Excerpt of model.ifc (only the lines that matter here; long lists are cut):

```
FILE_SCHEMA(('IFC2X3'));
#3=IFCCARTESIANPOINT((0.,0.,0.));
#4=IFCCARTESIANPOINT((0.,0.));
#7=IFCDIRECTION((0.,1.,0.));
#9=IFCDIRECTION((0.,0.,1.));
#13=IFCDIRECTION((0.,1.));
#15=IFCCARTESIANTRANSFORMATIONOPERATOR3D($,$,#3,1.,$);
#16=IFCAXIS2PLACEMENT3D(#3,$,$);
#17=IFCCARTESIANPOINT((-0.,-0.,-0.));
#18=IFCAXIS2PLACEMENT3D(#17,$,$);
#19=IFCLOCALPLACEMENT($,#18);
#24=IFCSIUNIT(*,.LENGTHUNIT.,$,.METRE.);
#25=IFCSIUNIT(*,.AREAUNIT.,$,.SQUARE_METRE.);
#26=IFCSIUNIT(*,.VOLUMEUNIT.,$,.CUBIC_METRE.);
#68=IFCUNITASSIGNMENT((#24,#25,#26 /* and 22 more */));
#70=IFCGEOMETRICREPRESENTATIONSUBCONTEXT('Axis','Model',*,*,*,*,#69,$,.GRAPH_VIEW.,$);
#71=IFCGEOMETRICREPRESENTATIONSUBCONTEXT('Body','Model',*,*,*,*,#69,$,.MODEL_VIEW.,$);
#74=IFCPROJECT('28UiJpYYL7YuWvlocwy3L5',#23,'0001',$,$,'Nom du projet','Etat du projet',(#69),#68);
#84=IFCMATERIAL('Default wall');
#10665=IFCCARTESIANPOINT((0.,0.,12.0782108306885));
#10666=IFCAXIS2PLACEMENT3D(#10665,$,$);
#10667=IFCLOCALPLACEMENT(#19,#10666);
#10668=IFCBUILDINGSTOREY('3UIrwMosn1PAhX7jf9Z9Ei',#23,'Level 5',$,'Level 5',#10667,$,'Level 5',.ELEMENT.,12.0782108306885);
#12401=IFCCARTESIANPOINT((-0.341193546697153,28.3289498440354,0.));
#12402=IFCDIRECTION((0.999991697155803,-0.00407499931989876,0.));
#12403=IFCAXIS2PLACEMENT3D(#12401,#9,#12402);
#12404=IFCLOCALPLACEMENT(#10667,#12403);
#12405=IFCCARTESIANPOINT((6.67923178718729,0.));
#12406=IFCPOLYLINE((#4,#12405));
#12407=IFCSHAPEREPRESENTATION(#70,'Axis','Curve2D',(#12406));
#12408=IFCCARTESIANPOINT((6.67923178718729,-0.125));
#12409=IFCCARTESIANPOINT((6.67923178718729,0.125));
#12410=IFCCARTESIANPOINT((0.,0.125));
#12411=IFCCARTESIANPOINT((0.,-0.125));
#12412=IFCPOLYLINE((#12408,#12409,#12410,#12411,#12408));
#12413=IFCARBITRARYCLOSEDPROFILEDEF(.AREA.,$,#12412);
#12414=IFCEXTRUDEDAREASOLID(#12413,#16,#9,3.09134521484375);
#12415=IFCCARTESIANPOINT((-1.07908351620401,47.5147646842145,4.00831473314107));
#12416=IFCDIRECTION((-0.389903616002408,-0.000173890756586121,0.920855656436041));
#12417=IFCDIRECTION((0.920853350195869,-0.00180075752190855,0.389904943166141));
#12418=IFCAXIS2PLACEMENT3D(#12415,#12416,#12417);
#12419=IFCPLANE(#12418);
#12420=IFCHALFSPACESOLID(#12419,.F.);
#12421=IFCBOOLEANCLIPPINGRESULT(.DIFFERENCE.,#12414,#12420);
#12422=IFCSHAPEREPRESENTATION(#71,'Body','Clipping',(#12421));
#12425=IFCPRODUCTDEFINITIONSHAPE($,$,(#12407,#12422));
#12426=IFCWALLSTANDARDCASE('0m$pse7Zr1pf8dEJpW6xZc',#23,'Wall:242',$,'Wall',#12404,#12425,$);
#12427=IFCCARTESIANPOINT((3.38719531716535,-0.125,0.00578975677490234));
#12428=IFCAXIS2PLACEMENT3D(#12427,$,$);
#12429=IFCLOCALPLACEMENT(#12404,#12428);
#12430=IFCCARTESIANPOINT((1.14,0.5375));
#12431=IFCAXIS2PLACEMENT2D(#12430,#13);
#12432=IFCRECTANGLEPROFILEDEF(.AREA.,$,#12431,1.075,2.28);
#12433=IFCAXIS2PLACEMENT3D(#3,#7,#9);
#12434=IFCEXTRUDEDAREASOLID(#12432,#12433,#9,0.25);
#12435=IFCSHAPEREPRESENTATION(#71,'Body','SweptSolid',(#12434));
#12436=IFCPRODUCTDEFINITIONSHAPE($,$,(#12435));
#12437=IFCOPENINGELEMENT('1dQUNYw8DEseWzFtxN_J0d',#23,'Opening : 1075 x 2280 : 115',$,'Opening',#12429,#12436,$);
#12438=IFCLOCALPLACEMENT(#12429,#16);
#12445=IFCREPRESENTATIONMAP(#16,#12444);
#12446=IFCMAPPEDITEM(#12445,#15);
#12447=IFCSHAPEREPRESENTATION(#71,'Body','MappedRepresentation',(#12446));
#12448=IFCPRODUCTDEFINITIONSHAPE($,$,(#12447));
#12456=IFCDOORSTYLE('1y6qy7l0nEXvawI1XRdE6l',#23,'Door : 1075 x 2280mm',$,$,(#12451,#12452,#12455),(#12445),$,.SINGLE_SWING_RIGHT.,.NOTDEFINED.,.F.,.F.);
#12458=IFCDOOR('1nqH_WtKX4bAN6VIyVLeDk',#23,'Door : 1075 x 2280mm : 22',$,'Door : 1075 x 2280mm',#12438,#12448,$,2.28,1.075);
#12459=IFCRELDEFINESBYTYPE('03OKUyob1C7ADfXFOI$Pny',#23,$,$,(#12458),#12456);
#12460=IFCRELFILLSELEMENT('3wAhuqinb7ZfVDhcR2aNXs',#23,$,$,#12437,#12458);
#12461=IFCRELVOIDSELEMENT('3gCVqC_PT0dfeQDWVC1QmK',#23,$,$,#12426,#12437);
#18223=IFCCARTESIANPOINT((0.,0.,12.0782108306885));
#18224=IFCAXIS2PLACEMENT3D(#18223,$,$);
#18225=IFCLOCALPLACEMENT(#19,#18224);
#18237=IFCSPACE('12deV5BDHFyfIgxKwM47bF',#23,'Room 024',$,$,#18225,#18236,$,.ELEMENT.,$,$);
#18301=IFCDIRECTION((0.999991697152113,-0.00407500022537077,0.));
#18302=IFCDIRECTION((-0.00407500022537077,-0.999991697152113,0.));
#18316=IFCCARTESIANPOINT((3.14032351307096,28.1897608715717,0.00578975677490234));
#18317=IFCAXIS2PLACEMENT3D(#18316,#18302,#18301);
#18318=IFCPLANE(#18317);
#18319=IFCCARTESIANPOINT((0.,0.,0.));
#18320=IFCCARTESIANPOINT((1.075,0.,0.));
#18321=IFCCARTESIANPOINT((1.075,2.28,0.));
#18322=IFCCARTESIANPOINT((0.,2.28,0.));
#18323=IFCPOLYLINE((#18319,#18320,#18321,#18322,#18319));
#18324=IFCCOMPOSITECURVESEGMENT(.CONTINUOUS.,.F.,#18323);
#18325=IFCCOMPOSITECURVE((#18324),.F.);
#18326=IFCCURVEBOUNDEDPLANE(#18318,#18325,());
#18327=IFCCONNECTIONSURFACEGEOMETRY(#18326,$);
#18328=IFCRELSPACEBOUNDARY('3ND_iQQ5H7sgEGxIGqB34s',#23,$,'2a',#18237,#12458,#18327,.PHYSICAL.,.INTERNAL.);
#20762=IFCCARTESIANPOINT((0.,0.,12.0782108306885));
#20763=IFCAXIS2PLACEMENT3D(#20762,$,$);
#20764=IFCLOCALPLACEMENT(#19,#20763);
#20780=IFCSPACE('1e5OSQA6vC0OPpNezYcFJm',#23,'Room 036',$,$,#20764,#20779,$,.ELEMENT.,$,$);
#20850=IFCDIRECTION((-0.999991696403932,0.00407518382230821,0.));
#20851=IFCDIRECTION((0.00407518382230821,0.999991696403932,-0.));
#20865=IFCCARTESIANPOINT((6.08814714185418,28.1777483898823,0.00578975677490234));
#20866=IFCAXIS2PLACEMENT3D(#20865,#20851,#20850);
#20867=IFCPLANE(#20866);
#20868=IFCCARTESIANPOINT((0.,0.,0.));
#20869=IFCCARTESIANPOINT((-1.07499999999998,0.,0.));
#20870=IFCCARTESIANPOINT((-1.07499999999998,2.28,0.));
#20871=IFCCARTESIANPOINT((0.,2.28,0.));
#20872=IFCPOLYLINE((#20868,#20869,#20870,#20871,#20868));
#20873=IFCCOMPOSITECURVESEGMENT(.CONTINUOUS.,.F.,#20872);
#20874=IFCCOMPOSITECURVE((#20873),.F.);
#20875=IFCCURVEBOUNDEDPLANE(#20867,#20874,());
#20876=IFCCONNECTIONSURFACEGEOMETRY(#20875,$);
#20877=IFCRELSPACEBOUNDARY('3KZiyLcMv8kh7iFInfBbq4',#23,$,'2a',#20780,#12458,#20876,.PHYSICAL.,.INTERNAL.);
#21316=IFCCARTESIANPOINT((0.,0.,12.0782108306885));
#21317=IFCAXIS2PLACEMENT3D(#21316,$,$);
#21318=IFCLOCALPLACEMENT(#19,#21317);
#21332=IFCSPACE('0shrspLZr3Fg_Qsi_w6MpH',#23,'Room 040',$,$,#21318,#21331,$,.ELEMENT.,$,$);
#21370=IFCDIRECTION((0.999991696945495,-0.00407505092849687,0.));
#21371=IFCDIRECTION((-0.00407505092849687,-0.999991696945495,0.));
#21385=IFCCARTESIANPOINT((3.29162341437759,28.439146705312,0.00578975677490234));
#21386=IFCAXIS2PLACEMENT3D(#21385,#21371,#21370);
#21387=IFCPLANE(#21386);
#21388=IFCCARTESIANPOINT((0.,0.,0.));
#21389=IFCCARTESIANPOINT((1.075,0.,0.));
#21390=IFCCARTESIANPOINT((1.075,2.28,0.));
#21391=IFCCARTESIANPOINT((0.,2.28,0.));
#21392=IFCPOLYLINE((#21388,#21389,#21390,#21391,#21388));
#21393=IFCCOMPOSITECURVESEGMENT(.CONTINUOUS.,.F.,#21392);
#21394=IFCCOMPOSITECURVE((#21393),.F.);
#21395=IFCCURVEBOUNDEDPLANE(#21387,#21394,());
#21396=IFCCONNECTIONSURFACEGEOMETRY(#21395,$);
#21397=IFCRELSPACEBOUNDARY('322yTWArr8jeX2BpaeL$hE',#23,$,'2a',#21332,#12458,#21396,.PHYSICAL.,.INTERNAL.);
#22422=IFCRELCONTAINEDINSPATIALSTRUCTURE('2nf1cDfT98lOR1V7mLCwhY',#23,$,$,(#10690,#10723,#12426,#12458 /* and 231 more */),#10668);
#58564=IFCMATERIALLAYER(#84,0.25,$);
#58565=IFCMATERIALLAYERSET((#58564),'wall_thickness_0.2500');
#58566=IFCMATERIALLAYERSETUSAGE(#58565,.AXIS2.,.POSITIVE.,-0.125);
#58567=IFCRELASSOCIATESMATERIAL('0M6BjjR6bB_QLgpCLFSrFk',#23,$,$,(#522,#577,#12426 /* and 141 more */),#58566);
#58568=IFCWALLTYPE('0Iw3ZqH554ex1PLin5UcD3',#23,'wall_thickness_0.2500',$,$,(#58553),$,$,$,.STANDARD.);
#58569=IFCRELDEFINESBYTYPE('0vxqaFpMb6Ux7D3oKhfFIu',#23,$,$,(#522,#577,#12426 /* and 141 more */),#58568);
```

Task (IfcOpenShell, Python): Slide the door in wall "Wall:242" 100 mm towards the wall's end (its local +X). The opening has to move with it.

```python
import numpy as np
import ifcopenshell
import ifcopenshell.api.geometry
import ifcopenshell.util.placement
import ifcopenshell.util.unit

model = ifcopenshell.open("model.ifc")
unit_scale = ifcopenshell.util.unit.calculate_unit_scale(model)

door = model.by_id(12458)
opening = door.FillsVoids[0].RelatingOpeningElement
wall = opening.VoidsElements[0].RelatingBuildingElement

wall_matrix = ifcopenshell.util.placement.get_local_placement(wall.ObjectPlacement)
shift = wall_matrix[:3, 0] * 0.1 / unit_scale
before = ifcopenshell.util.placement.get_local_placement(door.ObjectPlacement)[:3, 3].copy()

# The door is placed relative to its opening, so it follows when the opening moves.
matrix = ifcopenshell.util.placement.get_local_placement(opening.ObjectPlacement)
matrix[:3, 3] += shift
ifcopenshell.api.geometry.edit_object_placement(
    model, product=opening, matrix=matrix, is_si=False, should_transform_children=True
)

# Space boundary surfaces are stored in each space's coordinates; move them too.
for rel in door.ProvidesBoundaries:
    if not rel.ConnectionGeometry:
        continue
    surface = rel.ConnectionGeometry.SurfaceOnRelatingElement.BasisSurface
    space_matrix = ifcopenshell.util.placement.get_local_placement(rel.RelatingSpace.ObjectPlacement)
    point = np.array(surface.Position.Location.Coordinates) + space_matrix[:3, :3].T @ shift
    surface.Position = model.createIfcAxis2Placement3D(
        model.createIfcCartesianPoint(point.tolist()), surface.Position.Axis, surface.Position.RefDirection
    )

after = ifcopenshell.util.placement.get_local_placement(door.ObjectPlacement)[:3, 3]
print("door moved by", (after - before).round(3) + 0.0)

model.write("model_edited.ifc")
```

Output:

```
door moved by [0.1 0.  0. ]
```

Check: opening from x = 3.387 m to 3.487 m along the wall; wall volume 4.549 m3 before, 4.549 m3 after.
